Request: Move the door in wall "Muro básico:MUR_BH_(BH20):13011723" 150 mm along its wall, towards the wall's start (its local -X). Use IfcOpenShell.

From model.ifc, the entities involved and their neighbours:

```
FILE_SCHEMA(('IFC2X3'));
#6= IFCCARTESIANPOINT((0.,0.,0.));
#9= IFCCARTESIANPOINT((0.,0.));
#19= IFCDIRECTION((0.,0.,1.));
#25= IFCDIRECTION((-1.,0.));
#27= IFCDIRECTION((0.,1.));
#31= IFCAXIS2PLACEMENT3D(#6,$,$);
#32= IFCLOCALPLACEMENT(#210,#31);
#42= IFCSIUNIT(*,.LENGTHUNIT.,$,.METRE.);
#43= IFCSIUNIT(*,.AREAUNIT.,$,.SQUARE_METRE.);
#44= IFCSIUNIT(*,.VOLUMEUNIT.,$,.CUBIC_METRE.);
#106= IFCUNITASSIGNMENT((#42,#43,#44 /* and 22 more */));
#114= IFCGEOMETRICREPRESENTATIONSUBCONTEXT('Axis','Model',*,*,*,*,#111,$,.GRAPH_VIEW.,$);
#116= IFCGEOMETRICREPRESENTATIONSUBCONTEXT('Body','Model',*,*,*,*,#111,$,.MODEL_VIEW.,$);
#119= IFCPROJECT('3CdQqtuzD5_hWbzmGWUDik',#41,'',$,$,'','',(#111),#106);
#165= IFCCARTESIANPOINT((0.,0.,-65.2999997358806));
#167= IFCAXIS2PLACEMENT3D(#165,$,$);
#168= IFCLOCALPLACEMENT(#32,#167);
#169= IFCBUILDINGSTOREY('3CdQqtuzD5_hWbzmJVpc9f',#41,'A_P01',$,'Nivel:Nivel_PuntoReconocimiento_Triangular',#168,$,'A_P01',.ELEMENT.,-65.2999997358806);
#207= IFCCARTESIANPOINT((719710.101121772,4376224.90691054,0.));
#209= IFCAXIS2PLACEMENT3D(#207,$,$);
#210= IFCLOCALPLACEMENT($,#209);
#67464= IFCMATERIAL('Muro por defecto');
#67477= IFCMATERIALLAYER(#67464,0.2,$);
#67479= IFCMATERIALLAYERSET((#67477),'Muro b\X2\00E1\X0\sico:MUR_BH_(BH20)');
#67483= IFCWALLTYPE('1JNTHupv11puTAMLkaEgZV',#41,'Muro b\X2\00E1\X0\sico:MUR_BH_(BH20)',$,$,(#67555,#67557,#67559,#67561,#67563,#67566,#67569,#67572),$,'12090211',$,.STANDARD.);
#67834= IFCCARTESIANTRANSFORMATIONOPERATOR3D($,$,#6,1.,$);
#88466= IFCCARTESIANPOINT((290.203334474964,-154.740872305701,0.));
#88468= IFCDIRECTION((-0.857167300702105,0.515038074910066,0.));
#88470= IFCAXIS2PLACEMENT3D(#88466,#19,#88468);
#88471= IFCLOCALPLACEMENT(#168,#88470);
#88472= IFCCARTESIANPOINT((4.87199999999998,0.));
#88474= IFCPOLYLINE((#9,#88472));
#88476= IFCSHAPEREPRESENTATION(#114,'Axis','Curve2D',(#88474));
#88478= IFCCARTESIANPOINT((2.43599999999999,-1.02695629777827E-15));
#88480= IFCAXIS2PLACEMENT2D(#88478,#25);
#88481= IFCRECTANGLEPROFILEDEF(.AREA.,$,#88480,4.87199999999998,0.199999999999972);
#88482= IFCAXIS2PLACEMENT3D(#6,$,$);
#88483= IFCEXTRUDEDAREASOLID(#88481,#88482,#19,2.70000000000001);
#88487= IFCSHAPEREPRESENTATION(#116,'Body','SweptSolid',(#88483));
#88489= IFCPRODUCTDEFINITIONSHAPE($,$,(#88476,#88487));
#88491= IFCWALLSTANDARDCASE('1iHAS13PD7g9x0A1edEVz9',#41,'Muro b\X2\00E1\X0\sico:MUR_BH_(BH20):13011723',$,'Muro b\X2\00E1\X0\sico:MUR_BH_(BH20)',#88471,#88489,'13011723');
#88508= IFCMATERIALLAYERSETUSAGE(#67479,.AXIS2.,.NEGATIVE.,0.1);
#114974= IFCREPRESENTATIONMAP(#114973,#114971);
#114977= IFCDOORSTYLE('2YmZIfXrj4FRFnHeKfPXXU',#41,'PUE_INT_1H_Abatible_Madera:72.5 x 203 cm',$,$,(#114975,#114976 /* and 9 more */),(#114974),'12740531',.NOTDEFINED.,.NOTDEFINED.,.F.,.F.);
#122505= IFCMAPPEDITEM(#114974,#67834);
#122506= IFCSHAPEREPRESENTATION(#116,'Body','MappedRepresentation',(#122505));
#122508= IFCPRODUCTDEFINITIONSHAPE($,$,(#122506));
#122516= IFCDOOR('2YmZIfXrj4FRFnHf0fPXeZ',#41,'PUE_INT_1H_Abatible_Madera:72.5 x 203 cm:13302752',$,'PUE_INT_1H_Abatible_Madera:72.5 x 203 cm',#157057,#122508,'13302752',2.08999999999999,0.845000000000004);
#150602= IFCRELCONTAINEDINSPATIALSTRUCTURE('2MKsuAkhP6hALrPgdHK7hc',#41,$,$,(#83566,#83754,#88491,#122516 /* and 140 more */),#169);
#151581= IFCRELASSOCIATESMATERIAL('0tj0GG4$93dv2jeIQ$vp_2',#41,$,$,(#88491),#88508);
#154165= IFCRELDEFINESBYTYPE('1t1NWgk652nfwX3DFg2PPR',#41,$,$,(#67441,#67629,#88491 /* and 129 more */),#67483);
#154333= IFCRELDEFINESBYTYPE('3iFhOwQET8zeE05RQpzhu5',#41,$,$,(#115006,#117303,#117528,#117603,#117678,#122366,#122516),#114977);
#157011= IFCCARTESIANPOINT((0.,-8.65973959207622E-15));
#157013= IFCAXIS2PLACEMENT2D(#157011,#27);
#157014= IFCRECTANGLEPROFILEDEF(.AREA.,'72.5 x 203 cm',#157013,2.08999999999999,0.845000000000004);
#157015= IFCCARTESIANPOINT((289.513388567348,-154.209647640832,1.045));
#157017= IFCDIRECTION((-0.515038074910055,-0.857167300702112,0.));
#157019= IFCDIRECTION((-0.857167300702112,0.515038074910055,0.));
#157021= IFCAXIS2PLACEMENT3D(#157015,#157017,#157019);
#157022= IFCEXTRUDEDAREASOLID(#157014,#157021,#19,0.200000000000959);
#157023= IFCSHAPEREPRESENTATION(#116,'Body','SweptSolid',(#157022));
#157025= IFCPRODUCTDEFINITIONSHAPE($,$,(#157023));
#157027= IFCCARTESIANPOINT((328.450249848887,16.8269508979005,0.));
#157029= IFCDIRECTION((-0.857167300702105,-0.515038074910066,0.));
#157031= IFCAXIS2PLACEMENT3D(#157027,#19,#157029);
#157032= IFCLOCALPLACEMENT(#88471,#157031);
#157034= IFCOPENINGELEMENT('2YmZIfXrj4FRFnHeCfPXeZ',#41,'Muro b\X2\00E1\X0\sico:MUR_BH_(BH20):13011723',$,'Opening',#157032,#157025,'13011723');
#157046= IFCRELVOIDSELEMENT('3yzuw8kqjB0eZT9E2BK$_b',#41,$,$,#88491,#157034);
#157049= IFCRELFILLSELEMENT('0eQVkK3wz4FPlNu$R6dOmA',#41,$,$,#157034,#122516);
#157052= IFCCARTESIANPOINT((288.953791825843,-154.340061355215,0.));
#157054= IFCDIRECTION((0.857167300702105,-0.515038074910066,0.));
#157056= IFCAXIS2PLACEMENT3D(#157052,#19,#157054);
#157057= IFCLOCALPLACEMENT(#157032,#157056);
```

```python
import ifcopenshell
import ifcopenshell.api.geometry
import ifcopenshell.util.placement

model = ifcopenshell.open("model.ifc")

door = model.by_guid("2YmZIfXrj4FRFnHf0fPXeZ")
opening = door.FillsVoids[0].RelatingOpeningElement
wall = opening.VoidsElements[0].RelatingBuildingElement

wall_matrix = ifcopenshell.util.placement.get_local_placement(wall.ObjectPlacement)
shift = wall_matrix[:3, 0] * -0.15
before = ifcopenshell.util.placement.get_local_placement(door.ObjectPlacement)[:3, 3].copy()

# The door is placed relative to its opening, so it follows when the opening moves.
matrix = ifcopenshell.util.placement.get_local_placement(opening.ObjectPlacement)
matrix[:3, 3] += shift
ifcopenshell.api.geometry.edit_object_placement(
    model, product=opening, matrix=matrix, is_si=False, should_transform_children=True
)

after = ifcopenshell.util.placement.get_local_placement(door.ObjectPlacement)[:3, 3]
print("door moved by", (after - before).round(3) + 0.0)

model.write("model_rev.ifc")
```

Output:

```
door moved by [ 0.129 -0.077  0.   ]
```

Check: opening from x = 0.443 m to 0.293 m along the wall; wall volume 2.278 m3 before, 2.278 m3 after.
